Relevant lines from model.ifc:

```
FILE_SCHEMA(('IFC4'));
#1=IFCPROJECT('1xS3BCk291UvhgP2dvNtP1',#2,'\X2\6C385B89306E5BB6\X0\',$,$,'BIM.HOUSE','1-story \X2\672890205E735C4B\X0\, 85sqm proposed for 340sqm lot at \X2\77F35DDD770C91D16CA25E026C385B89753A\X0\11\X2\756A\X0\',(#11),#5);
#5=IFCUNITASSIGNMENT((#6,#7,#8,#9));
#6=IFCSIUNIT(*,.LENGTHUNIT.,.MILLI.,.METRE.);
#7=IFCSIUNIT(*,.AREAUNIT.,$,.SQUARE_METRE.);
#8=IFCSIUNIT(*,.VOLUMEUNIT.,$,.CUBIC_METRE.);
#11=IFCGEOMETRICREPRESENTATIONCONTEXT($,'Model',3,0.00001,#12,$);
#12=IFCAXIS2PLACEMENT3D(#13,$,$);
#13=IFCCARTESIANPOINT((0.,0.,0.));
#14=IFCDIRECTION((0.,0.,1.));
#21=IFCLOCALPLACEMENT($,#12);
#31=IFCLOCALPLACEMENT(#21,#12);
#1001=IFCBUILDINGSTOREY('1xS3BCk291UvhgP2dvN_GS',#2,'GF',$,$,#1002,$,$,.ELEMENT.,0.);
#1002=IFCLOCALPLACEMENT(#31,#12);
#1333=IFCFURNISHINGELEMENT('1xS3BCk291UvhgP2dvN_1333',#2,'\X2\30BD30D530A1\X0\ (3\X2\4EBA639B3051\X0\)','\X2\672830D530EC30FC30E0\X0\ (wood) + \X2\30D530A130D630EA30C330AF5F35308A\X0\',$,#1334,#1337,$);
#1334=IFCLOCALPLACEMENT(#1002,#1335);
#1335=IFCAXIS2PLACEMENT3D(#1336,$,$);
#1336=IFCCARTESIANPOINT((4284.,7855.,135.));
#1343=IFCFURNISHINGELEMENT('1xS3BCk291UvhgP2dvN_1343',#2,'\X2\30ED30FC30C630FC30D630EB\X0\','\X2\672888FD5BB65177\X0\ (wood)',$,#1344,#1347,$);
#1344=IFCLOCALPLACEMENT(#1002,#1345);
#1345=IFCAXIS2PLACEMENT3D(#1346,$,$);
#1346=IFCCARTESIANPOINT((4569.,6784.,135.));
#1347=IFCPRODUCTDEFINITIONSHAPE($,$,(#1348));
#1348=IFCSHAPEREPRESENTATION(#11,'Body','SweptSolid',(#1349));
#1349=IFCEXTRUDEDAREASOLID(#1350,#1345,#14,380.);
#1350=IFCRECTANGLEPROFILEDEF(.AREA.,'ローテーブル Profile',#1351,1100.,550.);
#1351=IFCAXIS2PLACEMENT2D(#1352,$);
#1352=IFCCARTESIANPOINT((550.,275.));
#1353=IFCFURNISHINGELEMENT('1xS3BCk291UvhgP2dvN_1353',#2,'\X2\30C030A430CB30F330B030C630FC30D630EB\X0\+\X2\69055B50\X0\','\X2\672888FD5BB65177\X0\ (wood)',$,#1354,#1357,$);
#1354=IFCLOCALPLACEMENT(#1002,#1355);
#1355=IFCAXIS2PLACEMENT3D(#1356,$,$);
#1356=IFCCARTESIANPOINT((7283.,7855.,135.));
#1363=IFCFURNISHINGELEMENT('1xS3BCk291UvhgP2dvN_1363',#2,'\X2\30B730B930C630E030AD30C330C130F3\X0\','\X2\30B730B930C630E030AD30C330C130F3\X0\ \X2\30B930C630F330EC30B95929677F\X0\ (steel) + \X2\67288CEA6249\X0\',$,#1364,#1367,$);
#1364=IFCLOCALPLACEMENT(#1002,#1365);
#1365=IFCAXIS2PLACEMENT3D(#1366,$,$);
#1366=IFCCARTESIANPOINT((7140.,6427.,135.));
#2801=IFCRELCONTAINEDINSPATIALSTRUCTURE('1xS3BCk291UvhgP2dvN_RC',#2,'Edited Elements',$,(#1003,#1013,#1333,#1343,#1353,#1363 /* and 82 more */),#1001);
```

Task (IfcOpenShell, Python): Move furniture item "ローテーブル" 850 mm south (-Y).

```python
import ifcopenshell
import ifcopenshell.api.geometry
import ifcopenshell.util.placement

model = ifcopenshell.open("model.ifc")

item = model.by_guid("1xS3BCk291UvhgP2dvN_1343")
matrix = ifcopenshell.util.placement.get_local_placement(item.ObjectPlacement)
matrix[1, 3] -= 850.0
ifcopenshell.api.geometry.edit_object_placement(model, product=item, matrix=matrix, is_si=False)

print(ifcopenshell.util.placement.get_local_placement(item.ObjectPlacement).round(3) + 0.0)

model.write("model_edited.ifc")
```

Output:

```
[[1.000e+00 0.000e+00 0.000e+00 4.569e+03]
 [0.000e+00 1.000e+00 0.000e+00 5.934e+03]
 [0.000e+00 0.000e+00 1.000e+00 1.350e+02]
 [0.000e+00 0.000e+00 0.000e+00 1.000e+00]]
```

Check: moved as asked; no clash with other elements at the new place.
